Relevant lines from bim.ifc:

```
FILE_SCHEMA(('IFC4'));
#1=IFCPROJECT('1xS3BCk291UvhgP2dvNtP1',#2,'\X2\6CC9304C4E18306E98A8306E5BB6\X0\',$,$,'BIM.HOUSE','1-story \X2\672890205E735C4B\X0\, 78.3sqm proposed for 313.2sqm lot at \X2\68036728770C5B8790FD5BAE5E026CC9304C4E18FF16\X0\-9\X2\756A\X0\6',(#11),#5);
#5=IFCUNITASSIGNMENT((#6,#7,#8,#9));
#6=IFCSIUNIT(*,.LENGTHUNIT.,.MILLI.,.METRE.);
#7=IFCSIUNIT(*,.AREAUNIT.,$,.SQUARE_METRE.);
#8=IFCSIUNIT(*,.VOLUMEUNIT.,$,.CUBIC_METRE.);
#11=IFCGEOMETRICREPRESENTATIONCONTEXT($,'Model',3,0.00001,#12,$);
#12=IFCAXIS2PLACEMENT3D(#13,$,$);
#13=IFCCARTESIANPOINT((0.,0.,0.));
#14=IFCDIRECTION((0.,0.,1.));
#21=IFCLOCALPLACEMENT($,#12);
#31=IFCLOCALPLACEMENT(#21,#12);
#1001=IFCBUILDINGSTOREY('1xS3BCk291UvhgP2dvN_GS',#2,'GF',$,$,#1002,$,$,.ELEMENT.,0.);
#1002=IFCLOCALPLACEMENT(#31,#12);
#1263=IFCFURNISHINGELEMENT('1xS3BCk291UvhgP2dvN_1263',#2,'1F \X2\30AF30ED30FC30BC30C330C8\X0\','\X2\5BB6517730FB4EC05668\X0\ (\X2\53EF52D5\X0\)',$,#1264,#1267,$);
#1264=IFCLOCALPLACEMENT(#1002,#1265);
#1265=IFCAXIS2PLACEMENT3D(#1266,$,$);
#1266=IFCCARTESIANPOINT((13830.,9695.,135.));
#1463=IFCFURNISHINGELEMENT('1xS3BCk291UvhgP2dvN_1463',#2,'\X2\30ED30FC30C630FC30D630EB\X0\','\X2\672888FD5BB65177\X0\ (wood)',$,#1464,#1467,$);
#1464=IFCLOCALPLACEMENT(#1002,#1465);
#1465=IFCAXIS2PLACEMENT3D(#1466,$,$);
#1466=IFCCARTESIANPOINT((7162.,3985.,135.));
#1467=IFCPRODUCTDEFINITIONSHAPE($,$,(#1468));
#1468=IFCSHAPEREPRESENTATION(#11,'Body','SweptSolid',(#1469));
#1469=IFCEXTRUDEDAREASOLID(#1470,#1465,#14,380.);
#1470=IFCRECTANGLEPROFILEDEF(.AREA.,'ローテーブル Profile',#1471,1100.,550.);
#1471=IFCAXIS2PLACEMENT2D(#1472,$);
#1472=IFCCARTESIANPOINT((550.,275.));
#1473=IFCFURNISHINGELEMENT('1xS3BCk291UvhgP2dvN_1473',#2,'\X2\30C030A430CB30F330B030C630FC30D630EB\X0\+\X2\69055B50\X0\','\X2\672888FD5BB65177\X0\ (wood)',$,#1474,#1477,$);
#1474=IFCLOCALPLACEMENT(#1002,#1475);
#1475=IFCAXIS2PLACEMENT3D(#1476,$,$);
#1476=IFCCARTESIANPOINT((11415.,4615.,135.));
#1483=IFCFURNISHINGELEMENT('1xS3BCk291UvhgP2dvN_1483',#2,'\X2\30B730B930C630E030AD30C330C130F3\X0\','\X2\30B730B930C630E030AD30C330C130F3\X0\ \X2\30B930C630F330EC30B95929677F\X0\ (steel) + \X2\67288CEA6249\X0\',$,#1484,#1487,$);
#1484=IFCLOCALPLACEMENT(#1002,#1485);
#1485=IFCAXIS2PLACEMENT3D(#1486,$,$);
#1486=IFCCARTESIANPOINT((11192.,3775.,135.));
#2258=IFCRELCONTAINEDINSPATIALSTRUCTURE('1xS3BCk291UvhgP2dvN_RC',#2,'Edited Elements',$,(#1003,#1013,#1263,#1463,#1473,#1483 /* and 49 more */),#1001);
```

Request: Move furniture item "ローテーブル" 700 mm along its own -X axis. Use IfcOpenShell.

```python
import ifcopenshell
import ifcopenshell.api.geometry
import ifcopenshell.util.placement
import ifcopenshell.util.unit

model = ifcopenshell.open("bim.ifc")
unit_scale = ifcopenshell.util.unit.calculate_unit_scale(model)

item = model.by_id(1463)
matrix = ifcopenshell.util.placement.get_local_placement(item.ObjectPlacement)
matrix[:3, 3] -= matrix[:3, 0] * 0.7 / unit_scale
ifcopenshell.api.geometry.edit_object_placement(model, product=item, matrix=matrix, is_si=False)

print(ifcopenshell.util.placement.get_local_placement(item.ObjectPlacement).round(3) + 0.0)

model.write("bim_rev.ifc")
```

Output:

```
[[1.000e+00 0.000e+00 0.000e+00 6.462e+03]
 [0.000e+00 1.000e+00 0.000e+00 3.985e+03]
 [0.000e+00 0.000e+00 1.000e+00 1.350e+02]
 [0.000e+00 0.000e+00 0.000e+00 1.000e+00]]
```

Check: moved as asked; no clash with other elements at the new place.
